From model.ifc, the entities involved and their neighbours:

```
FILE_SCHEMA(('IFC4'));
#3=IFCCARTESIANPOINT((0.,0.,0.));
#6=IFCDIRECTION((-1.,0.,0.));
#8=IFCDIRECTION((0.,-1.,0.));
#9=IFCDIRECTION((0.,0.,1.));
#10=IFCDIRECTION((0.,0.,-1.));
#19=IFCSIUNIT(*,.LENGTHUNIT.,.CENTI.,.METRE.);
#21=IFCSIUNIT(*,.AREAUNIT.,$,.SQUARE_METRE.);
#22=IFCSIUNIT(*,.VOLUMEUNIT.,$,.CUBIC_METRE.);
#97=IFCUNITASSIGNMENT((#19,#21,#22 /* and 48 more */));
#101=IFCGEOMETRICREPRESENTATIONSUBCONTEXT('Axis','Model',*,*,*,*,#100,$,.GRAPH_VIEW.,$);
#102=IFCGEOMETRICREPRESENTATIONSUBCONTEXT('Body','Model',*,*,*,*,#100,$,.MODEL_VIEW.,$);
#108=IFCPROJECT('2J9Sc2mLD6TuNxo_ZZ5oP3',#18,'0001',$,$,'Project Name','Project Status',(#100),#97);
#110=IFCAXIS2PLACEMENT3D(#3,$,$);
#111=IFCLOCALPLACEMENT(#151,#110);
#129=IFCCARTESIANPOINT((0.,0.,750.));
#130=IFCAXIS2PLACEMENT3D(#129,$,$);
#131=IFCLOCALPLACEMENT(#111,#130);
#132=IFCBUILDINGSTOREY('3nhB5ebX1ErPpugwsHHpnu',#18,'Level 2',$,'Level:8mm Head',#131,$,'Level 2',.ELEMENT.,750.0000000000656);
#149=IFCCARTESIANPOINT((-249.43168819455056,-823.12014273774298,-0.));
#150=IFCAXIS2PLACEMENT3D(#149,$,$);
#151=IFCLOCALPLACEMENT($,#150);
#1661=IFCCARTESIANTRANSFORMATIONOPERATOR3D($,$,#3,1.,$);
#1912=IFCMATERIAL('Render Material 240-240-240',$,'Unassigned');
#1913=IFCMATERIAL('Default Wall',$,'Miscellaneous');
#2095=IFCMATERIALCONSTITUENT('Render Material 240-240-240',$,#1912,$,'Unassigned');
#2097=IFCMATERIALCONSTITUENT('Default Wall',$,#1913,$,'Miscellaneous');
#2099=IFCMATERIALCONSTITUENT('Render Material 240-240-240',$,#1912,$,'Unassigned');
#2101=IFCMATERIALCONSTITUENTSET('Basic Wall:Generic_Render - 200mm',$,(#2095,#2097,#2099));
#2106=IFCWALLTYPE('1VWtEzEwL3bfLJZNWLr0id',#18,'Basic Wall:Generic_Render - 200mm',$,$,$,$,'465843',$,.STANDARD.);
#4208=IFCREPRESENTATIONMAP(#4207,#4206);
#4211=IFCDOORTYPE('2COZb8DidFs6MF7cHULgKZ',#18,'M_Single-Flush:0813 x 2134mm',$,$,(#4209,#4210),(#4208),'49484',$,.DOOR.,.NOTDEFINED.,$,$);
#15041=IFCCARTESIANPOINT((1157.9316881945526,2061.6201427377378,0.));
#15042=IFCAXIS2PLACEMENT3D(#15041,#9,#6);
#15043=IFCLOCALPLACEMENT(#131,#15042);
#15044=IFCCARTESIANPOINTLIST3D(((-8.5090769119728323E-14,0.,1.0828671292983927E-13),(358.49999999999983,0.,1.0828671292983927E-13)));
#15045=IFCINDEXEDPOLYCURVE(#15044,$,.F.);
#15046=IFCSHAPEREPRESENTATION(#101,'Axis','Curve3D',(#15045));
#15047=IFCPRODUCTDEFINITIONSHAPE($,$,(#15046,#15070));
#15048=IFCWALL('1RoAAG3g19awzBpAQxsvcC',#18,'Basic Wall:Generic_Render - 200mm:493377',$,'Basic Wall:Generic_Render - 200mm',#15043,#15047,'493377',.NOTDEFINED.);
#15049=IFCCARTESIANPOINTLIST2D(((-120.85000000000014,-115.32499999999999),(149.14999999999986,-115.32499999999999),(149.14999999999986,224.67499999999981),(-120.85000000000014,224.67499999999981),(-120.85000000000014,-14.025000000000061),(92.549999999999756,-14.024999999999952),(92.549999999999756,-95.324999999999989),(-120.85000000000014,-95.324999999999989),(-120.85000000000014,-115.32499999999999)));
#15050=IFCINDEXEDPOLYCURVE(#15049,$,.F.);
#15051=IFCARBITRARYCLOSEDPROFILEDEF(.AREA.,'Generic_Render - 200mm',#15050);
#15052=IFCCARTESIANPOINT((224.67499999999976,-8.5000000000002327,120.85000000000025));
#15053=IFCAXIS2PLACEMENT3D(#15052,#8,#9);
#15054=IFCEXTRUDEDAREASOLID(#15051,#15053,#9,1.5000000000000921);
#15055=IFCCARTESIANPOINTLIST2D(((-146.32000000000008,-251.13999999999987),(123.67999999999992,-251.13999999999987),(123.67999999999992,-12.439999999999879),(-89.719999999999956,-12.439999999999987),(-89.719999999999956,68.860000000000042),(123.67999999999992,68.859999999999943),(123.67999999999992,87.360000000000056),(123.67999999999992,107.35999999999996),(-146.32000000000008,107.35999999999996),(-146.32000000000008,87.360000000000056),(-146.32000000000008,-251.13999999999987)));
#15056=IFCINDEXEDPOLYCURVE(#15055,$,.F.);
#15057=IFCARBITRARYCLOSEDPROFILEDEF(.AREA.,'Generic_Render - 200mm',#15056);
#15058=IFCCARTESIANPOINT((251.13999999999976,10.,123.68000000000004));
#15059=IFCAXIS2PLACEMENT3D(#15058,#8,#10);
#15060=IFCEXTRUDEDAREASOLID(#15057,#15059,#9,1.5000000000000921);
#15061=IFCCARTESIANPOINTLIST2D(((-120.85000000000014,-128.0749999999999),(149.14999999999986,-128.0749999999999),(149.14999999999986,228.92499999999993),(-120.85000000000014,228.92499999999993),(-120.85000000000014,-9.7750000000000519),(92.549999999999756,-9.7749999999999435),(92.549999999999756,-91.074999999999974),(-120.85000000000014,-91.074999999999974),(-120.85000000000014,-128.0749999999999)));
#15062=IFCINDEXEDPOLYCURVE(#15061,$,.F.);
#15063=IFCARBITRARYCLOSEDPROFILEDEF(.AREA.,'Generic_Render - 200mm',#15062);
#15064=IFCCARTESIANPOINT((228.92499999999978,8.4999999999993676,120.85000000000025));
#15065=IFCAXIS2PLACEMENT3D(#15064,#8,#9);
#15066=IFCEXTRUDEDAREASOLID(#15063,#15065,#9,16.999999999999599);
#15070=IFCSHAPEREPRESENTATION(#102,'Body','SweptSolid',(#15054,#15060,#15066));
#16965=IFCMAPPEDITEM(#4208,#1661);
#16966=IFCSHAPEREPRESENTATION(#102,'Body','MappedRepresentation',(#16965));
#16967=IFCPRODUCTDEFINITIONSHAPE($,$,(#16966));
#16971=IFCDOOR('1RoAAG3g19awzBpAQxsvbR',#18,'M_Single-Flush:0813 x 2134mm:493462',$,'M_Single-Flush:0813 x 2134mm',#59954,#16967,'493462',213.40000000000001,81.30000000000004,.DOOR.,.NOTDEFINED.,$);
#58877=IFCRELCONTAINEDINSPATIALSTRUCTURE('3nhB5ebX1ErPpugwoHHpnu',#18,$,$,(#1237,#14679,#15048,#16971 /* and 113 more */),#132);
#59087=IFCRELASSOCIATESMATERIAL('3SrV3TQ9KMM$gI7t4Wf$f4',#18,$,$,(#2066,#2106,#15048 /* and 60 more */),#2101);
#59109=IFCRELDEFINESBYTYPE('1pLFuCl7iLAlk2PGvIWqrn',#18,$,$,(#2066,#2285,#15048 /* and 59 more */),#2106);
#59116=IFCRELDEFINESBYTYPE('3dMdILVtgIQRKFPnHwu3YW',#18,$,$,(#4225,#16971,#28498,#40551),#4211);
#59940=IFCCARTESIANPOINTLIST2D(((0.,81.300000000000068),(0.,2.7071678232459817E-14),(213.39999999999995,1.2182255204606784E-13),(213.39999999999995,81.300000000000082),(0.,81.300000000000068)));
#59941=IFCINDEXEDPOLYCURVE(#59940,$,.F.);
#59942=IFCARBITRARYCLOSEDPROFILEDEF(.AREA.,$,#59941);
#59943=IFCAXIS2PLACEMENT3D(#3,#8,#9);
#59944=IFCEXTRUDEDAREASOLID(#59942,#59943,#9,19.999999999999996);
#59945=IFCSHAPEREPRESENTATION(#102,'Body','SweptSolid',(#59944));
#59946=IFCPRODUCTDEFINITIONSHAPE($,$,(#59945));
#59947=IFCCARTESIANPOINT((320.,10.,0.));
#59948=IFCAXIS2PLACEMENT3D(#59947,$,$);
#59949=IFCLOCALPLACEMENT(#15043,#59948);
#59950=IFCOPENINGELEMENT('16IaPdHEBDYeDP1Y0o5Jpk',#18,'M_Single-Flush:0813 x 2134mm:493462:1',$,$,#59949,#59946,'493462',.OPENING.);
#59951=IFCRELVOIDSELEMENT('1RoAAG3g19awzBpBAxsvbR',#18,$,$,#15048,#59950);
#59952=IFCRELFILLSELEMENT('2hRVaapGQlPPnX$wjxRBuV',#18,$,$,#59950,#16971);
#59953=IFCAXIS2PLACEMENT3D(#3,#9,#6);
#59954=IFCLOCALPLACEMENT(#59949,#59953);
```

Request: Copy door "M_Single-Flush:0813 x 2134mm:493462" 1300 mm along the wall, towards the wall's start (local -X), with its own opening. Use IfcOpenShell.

```python
import ifcopenshell
import ifcopenshell.api.feature
import ifcopenshell.api.geometry
import ifcopenshell.api.root
import ifcopenshell.geom
import ifcopenshell.util.element
import ifcopenshell.util.placement
import ifcopenshell.util.shape
import ifcopenshell.util.unit

model = ifcopenshell.open("model.ifc")
unit_scale = ifcopenshell.util.unit.calculate_unit_scale(model)
settings = ifcopenshell.geom.settings()


def volume(element):
    """Net volume in cubic metres, openings subtracted."""
    shape = ifcopenshell.geom.create_shape(settings, element)
    return ifcopenshell.util.shape.get_volume(shape.geometry)


door = model.by_id(16971)
opening = door.FillsVoids[0].RelatingOpeningElement
wall = opening.VoidsElements[0].RelatingBuildingElement
before = volume(wall)
shift = ifcopenshell.util.placement.get_local_placement(wall.ObjectPlacement)[:3, 0] * -1.3 / unit_scale

# copy_class copies the void relationship, type, container and properties, but no geometry.
new_opening = ifcopenshell.api.root.copy_class(model, product=opening)
new_opening.Representation = ifcopenshell.util.element.copy_deep(
    model, opening.Representation, exclude=["IfcGeometricRepresentationContext", "IfcRepresentationMap"]
)
new_opening.Name = "M_Single-Flush:0813 x 2134mm"
new_opening.Tag = None
new_door = ifcopenshell.api.root.copy_class(model, product=door)
new_door.Representation = ifcopenshell.util.element.copy_deep(
    model, door.Representation, exclude=["IfcGeometricRepresentationContext", "IfcRepresentationMap"]
)
new_door.Name = "M_Single-Flush:0813 x 2134mm"
new_door.Tag = None
ifcopenshell.api.feature.add_filling(model, opening=new_opening, element=new_door)

for old, new in ((opening, new_opening), (door, new_door)):
    matrix = ifcopenshell.util.placement.get_local_placement(old.ObjectPlacement)
    matrix[:3, 3] += shift
    ifcopenshell.api.geometry.edit_object_placement(model, product=new, matrix=matrix, is_si=False)

after = volume(wall)

print(f"wall volume {before:.3f} -> {after:.3f} m3")

model.write("model-out.ifc")
```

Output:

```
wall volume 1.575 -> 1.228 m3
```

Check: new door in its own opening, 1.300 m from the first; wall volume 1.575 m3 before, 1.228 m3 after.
